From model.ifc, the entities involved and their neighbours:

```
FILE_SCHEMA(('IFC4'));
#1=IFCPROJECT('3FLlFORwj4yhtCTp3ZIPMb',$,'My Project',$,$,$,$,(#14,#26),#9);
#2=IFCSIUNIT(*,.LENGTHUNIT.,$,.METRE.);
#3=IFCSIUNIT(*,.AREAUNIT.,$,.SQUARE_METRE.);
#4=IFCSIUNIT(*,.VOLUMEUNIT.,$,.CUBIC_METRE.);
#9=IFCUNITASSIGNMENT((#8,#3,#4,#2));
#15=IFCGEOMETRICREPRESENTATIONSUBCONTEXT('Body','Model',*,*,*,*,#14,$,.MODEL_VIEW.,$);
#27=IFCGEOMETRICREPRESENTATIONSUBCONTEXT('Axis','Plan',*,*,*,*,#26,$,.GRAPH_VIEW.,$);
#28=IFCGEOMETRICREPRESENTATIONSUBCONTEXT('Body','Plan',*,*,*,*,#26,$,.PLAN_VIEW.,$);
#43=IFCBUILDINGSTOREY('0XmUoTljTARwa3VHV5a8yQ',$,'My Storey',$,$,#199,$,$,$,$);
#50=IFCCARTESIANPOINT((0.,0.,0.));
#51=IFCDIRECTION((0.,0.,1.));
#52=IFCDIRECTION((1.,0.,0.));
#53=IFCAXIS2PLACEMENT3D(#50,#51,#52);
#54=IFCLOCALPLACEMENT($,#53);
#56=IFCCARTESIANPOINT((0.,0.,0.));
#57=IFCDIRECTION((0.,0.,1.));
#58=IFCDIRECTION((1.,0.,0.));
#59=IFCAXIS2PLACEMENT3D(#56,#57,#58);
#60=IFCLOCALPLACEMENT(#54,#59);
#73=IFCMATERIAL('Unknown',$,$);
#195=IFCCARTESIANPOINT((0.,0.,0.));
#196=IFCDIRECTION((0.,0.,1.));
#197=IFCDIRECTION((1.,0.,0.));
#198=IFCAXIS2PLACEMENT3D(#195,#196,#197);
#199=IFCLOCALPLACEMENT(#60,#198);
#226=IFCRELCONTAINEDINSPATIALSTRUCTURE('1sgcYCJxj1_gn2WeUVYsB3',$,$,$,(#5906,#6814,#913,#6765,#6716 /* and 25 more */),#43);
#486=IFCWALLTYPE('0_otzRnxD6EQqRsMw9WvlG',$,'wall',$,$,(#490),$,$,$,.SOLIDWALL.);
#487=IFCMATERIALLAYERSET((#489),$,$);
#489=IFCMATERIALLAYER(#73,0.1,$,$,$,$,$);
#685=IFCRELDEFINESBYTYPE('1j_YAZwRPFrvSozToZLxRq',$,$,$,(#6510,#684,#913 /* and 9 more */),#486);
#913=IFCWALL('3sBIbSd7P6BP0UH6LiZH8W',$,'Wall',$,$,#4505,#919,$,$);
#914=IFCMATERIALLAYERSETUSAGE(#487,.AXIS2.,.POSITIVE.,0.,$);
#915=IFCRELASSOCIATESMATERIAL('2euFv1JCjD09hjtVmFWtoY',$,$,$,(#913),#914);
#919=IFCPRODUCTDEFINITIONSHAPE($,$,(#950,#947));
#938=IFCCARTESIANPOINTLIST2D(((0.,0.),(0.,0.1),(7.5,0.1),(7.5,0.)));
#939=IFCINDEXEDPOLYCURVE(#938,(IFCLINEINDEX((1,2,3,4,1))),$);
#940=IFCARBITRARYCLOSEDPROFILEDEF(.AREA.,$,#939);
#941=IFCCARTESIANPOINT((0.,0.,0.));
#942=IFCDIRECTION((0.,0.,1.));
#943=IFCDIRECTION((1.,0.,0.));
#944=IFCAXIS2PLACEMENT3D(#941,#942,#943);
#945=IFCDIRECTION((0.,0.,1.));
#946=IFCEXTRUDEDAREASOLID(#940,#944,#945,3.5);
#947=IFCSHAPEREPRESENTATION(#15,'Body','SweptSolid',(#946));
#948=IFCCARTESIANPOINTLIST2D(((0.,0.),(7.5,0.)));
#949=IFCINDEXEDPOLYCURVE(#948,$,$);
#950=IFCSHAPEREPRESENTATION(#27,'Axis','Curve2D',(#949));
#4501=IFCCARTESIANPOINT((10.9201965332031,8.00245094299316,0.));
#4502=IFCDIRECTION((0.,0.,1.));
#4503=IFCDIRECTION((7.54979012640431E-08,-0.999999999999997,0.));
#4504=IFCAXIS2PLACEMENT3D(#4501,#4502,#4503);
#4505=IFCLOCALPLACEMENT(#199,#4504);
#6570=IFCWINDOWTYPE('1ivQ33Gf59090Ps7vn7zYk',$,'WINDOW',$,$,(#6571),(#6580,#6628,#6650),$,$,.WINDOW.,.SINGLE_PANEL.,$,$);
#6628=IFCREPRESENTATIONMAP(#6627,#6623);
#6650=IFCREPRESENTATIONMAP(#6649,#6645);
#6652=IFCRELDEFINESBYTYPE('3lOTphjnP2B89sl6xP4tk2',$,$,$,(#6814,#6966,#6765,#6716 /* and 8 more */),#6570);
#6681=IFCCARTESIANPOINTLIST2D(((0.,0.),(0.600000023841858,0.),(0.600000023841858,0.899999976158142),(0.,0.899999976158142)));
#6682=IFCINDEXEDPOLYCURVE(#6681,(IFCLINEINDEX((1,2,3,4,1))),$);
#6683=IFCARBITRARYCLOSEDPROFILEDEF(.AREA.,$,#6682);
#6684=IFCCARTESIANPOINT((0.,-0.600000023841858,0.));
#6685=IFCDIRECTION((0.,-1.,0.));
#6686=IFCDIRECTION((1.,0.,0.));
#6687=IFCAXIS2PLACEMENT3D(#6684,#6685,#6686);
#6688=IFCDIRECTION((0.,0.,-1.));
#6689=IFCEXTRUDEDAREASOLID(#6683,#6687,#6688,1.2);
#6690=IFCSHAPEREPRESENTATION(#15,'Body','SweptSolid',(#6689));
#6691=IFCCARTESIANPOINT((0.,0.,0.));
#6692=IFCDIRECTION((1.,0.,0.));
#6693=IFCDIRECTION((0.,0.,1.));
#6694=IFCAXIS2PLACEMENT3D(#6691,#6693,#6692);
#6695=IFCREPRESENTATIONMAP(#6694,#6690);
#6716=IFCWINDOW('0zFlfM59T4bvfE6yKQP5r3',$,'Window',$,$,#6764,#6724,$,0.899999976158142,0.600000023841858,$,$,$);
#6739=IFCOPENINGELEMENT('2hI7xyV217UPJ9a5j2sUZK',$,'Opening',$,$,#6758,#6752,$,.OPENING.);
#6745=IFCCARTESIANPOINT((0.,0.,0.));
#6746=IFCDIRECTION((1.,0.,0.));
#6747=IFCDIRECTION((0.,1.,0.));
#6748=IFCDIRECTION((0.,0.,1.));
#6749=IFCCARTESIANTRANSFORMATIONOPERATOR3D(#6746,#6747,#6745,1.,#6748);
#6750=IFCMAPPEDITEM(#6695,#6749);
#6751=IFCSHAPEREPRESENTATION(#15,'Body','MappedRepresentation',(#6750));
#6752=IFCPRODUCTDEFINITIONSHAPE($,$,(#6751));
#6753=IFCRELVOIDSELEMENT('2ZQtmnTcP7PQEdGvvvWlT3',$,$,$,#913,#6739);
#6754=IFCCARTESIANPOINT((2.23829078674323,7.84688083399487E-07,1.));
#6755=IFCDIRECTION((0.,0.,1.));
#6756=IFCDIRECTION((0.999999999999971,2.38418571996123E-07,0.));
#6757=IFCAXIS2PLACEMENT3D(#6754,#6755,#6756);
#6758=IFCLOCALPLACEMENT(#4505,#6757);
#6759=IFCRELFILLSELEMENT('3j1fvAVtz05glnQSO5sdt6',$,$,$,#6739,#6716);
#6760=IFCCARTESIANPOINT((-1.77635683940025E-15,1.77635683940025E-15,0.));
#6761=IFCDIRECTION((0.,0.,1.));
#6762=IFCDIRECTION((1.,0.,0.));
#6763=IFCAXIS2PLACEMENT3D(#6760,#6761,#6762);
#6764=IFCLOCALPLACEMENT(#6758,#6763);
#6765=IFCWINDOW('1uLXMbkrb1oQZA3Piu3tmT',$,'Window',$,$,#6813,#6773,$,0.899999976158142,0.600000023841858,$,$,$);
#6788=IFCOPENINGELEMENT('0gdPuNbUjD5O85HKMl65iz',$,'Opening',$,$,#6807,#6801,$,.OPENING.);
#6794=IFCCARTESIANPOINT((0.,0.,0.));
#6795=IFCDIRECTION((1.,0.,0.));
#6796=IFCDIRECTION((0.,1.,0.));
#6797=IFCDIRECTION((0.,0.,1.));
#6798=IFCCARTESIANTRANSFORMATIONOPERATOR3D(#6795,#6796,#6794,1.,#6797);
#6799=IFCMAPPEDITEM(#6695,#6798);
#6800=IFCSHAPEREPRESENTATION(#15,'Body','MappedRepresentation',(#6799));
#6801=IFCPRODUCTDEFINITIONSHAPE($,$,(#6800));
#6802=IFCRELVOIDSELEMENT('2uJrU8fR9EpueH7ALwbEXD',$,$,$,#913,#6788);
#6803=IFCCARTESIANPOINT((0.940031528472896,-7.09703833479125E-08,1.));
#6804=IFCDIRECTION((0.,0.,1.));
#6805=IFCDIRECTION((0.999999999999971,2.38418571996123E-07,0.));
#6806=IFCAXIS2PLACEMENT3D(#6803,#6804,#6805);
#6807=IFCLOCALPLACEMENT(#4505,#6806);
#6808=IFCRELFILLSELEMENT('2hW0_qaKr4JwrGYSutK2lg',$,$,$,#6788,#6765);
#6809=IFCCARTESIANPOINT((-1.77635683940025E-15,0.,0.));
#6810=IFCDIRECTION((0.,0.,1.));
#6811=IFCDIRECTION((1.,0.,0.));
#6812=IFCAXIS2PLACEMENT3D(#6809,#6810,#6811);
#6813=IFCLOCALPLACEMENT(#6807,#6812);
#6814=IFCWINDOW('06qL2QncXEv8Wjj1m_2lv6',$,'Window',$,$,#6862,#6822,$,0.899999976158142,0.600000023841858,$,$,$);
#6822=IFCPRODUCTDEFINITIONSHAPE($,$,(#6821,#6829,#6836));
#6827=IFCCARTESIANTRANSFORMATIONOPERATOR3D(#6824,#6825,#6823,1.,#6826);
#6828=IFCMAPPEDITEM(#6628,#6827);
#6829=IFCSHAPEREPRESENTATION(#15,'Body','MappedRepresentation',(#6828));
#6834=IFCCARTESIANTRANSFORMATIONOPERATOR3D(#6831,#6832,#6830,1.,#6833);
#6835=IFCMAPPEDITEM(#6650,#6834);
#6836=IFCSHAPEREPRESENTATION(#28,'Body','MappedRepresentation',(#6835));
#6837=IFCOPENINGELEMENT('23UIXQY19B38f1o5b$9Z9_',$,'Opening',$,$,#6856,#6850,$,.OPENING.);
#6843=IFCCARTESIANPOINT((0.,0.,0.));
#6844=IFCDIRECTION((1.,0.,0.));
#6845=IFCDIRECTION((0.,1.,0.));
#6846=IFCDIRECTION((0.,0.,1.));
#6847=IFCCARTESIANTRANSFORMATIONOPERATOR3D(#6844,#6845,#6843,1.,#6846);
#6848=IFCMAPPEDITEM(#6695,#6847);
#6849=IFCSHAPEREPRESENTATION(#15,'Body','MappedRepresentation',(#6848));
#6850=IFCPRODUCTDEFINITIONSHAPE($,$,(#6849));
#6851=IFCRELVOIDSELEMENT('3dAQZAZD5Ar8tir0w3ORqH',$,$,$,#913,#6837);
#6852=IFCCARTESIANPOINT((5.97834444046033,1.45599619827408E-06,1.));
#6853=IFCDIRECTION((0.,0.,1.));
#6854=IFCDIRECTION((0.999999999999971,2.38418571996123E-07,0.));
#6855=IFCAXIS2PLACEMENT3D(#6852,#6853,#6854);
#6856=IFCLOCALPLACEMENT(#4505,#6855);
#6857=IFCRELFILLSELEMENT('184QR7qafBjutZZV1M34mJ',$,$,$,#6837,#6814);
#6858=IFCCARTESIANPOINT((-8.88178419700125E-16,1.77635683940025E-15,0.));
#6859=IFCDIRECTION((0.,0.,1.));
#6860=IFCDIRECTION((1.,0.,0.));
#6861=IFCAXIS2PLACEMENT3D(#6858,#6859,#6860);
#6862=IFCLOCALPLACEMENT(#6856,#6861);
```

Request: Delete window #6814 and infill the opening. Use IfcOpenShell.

```python
import ifcopenshell
import ifcopenshell.api.feature
import ifcopenshell.api.root
import ifcopenshell.geom
import ifcopenshell.util.shape

model = ifcopenshell.open("model.ifc")
settings = ifcopenshell.geom.settings()


def volume(element):
    """Net volume in cubic metres, openings subtracted."""
    shape = ifcopenshell.geom.create_shape(settings, element)
    return ifcopenshell.util.shape.get_volume(shape.geometry)


window = model.by_guid("06qL2QncXEv8Wjj1m_2lv6")
opening = window.FillsVoids[0].RelatingOpeningElement
wall = opening.VoidsElements[0].RelatingBuildingElement
before = volume(wall)

ifcopenshell.api.root.remove_product(model, product=window)
ifcopenshell.api.feature.remove_feature(model, feature=opening)

after = volume(wall)

print(f"wall volume {before:.3f} -> {after:.3f} m3")

model.write("model_edited.ifc")
```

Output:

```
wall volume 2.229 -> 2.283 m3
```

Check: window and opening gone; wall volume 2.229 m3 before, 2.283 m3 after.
